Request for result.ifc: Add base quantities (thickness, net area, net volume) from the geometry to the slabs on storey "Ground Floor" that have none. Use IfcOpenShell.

First a look at what the model holds.

```python
import ifcopenshell
import ifcopenshell.util.element
import ifcopenshell.util.unit

model = ifcopenshell.open("result.ifc")
print(model.schema)
for unit_type in ("LENGTHUNIT", "AREAUNIT", "VOLUMEUNIT"):
    print(unit_type, ifcopenshell.util.unit.calculate_unit_scale(model, unit_type))
storey = next(s for s in model.by_type("IfcBuildingStorey") if s.Name == "Ground Floor")
slabs = [e for e in ifcopenshell.util.element.get_decomposition(storey) if e.is_a("IfcSlab")]
for e in sorted(slabs, key=lambda e: e.id()):
    print(e.id(), e.is_a(), e.Name, list(ifcopenshell.util.element.get_psets(e, qtos_only=True)), sep=" | ")
```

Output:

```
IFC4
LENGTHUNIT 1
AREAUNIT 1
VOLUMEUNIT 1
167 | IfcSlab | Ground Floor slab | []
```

```python
import ifcopenshell
import ifcopenshell.api.pset
import ifcopenshell.geom
import ifcopenshell.util.element
import ifcopenshell.util.shape
import ifcopenshell.util.unit

model = ifcopenshell.open("result.ifc")
unit_scale = ifcopenshell.util.unit.calculate_unit_scale(model)
area_scale = ifcopenshell.util.unit.calculate_unit_scale(model, "AREAUNIT")
volume_scale = ifcopenshell.util.unit.calculate_unit_scale(model, "VOLUMEUNIT")
settings = ifcopenshell.geom.settings()

storey = next(s for s in model.by_type("IfcBuildingStorey") if s.Name == "Ground Floor")
slabs = [e for e in ifcopenshell.util.element.get_decomposition(storey) if e.is_a("IfcSlab")]

for e in sorted(slabs, key=lambda e: e.id()):
    if ifcopenshell.util.element.get_psets(e, qtos_only=True, should_inherit=False):
        continue
    # Geometry comes back in metres, in the element's own axes.
    shape = ifcopenshell.geom.create_shape(settings, e)
    values = {
        "Width": ifcopenshell.util.shape.get_z(shape.geometry) / unit_scale,
        "NetArea": ifcopenshell.util.shape.get_footprint_area(shape.geometry) / area_scale,
        "NetVolume": ifcopenshell.util.shape.get_volume(shape.geometry) / volume_scale,
    }
    qto = ifcopenshell.api.pset.add_qto(model, product=e, name="Qto_SlabBaseQuantities")
    ifcopenshell.api.pset.edit_qto(model, qto=qto, properties=values)
    print(e.id(), {k: round(v, 3) for k, v in values.items()})

model.write("result_v2.ifc")
```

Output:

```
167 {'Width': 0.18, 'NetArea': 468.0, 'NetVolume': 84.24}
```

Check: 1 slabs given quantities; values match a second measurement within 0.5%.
